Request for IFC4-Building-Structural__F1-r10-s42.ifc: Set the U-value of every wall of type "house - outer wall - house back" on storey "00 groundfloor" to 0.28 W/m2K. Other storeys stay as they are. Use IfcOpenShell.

First a look at what the model holds.

```python
import ifcopenshell
import ifcopenshell.util.element

model = ifcopenshell.open("IFC4-Building-Structural__F1-r10-s42.ifc")
print(model.schema)
storey = next(s for s in model.by_type("IfcBuildingStorey") if s.Name == "00 groundfloor")
walls = [e for e in ifcopenshell.util.element.get_decomposition(storey) if e.is_a("IfcWall")]
seen = {}
for e in walls:
    element_type = ifcopenshell.util.element.get_type(e)
    key = (element_type.Name if element_type != e and element_type else None, ifcopenshell.util.element.get_pset(e, "Pset_WallCommon", "ThermalTransmittance"))
    seen[key] = seen.get(key, 0) + 1
for (name, value), count in sorted(seen.items(), key=str):
    print(count, "x", name, "|", value)
```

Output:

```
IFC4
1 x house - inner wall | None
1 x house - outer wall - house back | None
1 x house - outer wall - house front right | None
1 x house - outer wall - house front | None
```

```python
import ifcopenshell
import ifcopenshell.api.pset
import ifcopenshell.util.element

model = ifcopenshell.open("IFC4-Building-Structural__F1-r10-s42.ifc")

storey = next(s for s in model.by_type("IfcBuildingStorey") if s.Name == "00 groundfloor")
walls = [e for e in ifcopenshell.util.element.get_decomposition(storey) if e.is_a("IfcWall")]

count = 0
for e in walls:
    element_type = ifcopenshell.util.element.get_type(e)
    if element_type in (None, e) or element_type.Name != "house - outer wall - house back":
        continue
    # add_pset returns the element's existing set when there is one.
    pset = ifcopenshell.api.pset.add_pset(model, product=e, name="Pset_WallCommon")
    ifcopenshell.api.pset.edit_pset(model, pset=pset, properties={"ThermalTransmittance": 0.28})
    count += 1

print(count, "walls updated")

model.write("IFC4-Building-Structural__F1-r10-s42_edited.ifc")
```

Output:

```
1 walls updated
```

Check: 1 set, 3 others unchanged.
